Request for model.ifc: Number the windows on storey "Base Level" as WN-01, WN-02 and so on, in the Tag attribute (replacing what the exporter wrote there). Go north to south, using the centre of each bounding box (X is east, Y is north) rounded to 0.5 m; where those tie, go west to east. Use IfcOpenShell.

First a look at what the model holds.

```python
import ifcopenshell
import ifcopenshell.util.element
import ifcopenshell.util.placement

model = ifcopenshell.open("model.ifc")
print(model.schema)
storey = next(s for s in model.by_type("IfcBuildingStorey") if s.Name == "Base Level")
windows = [e for e in ifcopenshell.util.element.get_decomposition(storey) if e.is_a("IfcWindow")]
for e in sorted(windows, key=lambda e: e.id()):
    origin = ifcopenshell.util.placement.get_local_placement(e.ObjectPlacement)[:3, 3]
    print(e.id(), e.Tag, e.Name, origin.round(2) + 0.0, sep=" | ")
```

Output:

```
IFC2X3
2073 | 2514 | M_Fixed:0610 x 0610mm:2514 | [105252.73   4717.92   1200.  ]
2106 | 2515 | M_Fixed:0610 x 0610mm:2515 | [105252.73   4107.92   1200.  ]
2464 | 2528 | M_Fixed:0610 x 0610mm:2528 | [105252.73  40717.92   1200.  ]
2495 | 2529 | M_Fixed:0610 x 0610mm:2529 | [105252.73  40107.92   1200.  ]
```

```python
import ifcopenshell
import ifcopenshell.geom
import ifcopenshell.util.element
import ifcopenshell.util.shape

model = ifcopenshell.open("model.ifc")
settings = ifcopenshell.geom.settings()
settings.set("use-world-coords", True)


def centre(element):
    shape = ifcopenshell.geom.create_shape(settings, element)
    return ifcopenshell.util.shape.get_bbox_centroid(shape.geometry)


storey = next(s for s in model.by_type("IfcBuildingStorey") if s.Name == "Base Level")
windows = [e for e in ifcopenshell.util.element.get_decomposition(storey) if e.is_a("IfcWindow")]

# Insertion points can sit at a corner or the storey origin, so sort by the geometry (in metres).
centres = {e: centre(e) for e in windows}
windows.sort(key=lambda e: (-round(centres[e][1] / 0.5), centres[e][0]))

for i, e in enumerate(windows, start=1):
    number = f"WN-{i:02d}"
    e.Tag = number
    print(e.id(), number)

model.write("model-out.ifc")
```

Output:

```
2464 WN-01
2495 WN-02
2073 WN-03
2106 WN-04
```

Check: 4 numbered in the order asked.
